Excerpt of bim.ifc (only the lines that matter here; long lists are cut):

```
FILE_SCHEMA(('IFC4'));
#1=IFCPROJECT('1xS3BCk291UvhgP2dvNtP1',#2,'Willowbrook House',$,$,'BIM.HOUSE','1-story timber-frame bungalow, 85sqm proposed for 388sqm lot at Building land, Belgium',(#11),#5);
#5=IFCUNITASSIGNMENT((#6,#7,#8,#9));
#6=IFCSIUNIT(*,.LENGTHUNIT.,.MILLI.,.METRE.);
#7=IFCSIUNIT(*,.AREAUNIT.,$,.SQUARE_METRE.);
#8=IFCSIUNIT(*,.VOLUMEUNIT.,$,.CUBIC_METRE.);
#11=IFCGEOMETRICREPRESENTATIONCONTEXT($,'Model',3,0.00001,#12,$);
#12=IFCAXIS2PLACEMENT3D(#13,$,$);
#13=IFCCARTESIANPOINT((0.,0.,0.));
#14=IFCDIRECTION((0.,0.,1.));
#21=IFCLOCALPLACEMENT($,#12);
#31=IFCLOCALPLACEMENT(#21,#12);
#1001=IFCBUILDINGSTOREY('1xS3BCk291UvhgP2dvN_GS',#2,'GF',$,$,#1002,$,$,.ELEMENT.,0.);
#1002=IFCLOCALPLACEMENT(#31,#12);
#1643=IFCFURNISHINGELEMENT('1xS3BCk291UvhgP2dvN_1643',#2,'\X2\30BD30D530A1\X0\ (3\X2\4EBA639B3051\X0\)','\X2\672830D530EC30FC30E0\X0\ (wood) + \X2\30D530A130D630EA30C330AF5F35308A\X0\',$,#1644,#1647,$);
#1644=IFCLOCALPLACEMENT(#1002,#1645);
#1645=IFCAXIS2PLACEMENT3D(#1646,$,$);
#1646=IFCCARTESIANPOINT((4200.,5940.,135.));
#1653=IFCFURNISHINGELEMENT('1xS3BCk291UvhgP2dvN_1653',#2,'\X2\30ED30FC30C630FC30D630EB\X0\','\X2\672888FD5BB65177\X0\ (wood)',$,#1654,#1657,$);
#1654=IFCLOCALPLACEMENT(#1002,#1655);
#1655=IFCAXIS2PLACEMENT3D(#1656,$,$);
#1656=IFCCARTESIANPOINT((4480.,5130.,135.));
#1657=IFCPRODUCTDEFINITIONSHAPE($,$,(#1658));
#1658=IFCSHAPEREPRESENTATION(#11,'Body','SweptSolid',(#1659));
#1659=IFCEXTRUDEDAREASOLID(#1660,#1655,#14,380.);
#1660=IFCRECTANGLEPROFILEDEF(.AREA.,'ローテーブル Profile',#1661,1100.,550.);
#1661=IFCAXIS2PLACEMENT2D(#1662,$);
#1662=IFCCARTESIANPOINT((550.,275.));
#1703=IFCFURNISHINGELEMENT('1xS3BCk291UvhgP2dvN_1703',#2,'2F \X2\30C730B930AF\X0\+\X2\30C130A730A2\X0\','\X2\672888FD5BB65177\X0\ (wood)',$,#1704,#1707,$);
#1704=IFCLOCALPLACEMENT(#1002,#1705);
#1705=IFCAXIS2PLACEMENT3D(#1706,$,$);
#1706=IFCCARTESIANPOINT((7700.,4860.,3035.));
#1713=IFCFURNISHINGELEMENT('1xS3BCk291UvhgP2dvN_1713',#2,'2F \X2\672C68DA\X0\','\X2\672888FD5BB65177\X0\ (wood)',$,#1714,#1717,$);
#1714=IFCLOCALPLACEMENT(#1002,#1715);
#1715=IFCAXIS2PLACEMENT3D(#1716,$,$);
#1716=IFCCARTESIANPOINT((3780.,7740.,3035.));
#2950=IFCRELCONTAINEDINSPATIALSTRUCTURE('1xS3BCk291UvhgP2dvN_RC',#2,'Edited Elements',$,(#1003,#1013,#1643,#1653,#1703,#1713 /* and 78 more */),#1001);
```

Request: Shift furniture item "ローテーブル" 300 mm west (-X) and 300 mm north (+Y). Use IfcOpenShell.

```python
import ifcopenshell
import ifcopenshell.api.geometry
import ifcopenshell.util.placement
import ifcopenshell.util.unit

model = ifcopenshell.open("bim.ifc")
unit_scale = ifcopenshell.util.unit.calculate_unit_scale(model)

item = model.by_guid("1xS3BCk291UvhgP2dvN_1653")
matrix = ifcopenshell.util.placement.get_local_placement(item.ObjectPlacement)
matrix[0, 3] -= 0.3 / unit_scale
matrix[1, 3] += 0.3 / unit_scale
ifcopenshell.api.geometry.edit_object_placement(model, product=item, matrix=matrix, is_si=False)

print(ifcopenshell.util.placement.get_local_placement(item.ObjectPlacement).round(3) + 0.0)

model.write("bim_v2.ifc")
```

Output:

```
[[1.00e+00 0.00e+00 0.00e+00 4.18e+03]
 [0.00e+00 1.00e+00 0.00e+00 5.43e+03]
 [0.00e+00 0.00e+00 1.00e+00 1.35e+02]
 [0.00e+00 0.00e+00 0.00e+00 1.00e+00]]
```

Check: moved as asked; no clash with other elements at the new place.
